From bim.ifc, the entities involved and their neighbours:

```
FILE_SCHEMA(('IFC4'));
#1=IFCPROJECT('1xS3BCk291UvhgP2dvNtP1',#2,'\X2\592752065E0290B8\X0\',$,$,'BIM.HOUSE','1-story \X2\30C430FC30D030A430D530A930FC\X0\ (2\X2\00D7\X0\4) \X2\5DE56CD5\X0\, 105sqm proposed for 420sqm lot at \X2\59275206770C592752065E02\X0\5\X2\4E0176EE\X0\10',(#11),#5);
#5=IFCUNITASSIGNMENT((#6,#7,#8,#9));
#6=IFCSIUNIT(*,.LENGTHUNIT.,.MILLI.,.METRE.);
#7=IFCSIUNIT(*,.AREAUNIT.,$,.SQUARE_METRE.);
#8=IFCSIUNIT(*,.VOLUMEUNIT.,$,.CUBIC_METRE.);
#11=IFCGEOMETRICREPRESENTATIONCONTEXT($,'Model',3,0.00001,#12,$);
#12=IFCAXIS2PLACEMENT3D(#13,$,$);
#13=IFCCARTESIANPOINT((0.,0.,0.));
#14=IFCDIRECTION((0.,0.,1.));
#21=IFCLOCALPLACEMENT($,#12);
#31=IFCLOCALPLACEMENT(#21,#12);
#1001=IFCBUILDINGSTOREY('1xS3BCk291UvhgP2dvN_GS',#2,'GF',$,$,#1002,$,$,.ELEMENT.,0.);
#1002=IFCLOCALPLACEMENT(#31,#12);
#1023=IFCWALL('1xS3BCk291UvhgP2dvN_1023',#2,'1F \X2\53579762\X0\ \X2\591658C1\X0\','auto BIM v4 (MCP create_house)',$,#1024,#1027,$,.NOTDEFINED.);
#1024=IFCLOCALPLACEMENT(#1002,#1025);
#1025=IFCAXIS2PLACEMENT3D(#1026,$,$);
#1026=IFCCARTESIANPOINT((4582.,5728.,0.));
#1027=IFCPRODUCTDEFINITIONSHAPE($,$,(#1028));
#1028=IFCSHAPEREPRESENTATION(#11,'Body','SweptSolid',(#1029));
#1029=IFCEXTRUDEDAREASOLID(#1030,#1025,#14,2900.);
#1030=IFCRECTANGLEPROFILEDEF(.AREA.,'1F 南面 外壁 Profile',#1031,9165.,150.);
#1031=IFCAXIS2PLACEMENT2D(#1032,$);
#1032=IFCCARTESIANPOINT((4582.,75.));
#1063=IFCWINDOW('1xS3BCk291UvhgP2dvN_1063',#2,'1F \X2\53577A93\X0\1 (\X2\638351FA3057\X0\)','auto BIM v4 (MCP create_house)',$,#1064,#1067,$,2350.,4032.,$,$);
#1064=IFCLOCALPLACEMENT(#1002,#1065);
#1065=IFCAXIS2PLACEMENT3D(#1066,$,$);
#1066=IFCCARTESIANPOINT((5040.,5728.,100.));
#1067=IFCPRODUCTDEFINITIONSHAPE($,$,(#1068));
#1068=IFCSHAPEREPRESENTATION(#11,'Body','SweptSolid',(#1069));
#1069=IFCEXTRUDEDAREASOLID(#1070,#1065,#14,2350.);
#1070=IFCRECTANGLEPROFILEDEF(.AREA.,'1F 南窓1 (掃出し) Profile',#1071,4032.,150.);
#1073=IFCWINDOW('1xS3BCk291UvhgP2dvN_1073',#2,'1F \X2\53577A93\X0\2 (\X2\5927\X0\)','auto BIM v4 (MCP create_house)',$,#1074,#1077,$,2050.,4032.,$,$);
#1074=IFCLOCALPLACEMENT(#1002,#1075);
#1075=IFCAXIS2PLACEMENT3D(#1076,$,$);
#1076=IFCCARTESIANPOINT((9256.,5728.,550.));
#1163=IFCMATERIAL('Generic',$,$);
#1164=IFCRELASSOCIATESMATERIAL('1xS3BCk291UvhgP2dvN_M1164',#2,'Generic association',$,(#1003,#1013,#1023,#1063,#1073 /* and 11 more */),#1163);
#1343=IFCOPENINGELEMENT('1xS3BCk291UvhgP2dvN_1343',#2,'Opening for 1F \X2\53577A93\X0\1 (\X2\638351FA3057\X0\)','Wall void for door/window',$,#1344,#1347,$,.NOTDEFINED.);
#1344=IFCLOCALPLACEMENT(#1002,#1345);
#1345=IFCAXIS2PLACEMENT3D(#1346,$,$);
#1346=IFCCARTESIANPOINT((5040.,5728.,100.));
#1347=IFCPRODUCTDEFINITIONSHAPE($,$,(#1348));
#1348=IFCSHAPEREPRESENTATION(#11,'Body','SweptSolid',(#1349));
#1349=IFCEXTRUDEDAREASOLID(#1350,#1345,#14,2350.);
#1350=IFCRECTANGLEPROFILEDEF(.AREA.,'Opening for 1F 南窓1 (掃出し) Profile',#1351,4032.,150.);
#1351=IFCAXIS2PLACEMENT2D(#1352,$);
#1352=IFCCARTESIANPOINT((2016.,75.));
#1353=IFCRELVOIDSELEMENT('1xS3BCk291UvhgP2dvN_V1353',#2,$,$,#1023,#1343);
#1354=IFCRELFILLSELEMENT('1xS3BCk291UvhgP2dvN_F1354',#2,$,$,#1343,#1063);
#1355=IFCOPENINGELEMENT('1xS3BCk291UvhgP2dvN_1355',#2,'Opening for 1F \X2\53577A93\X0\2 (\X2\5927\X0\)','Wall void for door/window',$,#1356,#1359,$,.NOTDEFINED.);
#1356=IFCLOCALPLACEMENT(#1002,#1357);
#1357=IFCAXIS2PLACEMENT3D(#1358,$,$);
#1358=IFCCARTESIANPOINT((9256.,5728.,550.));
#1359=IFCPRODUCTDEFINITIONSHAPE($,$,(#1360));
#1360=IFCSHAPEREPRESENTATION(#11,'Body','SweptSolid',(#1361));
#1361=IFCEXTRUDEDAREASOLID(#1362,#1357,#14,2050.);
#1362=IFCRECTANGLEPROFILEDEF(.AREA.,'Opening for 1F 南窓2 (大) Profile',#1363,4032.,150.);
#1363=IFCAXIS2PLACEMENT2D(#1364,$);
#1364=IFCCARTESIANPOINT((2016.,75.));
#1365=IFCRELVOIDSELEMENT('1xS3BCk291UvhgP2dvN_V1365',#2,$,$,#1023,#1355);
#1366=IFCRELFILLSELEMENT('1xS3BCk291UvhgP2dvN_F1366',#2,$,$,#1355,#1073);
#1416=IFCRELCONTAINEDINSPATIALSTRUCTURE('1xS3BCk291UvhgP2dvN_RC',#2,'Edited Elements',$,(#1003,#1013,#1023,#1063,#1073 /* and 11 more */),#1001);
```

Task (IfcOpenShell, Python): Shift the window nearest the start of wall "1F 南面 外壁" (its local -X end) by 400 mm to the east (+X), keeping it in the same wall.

```python
import ifcopenshell
import ifcopenshell.api.geometry
import ifcopenshell.util.placement

model = ifcopenshell.open("bim.ifc")

window = model.by_guid("1xS3BCk291UvhgP2dvN_1063")
opening = window.FillsVoids[0].RelatingOpeningElement
wall = opening.VoidsElements[0].RelatingBuildingElement

wall_matrix = ifcopenshell.util.placement.get_local_placement(wall.ObjectPlacement)
shift = wall_matrix[:3, 0] * 400.0
before = ifcopenshell.util.placement.get_local_placement(window.ObjectPlacement)[:3, 3].copy()

# The window is not placed relative to its opening, so move both.
for product in (opening, window):
    matrix = ifcopenshell.util.placement.get_local_placement(product.ObjectPlacement)
    matrix[:3, 3] += shift
    ifcopenshell.api.geometry.edit_object_placement(model, product=product, matrix=matrix, is_si=False)

after = ifcopenshell.util.placement.get_local_placement(window.ObjectPlacement)[:3, 3]
print("window moved by", (after - before).round(3) + 0.0)

model.write("bim_v2.ifc")
```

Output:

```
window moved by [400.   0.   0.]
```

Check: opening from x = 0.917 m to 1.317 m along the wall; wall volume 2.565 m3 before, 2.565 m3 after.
